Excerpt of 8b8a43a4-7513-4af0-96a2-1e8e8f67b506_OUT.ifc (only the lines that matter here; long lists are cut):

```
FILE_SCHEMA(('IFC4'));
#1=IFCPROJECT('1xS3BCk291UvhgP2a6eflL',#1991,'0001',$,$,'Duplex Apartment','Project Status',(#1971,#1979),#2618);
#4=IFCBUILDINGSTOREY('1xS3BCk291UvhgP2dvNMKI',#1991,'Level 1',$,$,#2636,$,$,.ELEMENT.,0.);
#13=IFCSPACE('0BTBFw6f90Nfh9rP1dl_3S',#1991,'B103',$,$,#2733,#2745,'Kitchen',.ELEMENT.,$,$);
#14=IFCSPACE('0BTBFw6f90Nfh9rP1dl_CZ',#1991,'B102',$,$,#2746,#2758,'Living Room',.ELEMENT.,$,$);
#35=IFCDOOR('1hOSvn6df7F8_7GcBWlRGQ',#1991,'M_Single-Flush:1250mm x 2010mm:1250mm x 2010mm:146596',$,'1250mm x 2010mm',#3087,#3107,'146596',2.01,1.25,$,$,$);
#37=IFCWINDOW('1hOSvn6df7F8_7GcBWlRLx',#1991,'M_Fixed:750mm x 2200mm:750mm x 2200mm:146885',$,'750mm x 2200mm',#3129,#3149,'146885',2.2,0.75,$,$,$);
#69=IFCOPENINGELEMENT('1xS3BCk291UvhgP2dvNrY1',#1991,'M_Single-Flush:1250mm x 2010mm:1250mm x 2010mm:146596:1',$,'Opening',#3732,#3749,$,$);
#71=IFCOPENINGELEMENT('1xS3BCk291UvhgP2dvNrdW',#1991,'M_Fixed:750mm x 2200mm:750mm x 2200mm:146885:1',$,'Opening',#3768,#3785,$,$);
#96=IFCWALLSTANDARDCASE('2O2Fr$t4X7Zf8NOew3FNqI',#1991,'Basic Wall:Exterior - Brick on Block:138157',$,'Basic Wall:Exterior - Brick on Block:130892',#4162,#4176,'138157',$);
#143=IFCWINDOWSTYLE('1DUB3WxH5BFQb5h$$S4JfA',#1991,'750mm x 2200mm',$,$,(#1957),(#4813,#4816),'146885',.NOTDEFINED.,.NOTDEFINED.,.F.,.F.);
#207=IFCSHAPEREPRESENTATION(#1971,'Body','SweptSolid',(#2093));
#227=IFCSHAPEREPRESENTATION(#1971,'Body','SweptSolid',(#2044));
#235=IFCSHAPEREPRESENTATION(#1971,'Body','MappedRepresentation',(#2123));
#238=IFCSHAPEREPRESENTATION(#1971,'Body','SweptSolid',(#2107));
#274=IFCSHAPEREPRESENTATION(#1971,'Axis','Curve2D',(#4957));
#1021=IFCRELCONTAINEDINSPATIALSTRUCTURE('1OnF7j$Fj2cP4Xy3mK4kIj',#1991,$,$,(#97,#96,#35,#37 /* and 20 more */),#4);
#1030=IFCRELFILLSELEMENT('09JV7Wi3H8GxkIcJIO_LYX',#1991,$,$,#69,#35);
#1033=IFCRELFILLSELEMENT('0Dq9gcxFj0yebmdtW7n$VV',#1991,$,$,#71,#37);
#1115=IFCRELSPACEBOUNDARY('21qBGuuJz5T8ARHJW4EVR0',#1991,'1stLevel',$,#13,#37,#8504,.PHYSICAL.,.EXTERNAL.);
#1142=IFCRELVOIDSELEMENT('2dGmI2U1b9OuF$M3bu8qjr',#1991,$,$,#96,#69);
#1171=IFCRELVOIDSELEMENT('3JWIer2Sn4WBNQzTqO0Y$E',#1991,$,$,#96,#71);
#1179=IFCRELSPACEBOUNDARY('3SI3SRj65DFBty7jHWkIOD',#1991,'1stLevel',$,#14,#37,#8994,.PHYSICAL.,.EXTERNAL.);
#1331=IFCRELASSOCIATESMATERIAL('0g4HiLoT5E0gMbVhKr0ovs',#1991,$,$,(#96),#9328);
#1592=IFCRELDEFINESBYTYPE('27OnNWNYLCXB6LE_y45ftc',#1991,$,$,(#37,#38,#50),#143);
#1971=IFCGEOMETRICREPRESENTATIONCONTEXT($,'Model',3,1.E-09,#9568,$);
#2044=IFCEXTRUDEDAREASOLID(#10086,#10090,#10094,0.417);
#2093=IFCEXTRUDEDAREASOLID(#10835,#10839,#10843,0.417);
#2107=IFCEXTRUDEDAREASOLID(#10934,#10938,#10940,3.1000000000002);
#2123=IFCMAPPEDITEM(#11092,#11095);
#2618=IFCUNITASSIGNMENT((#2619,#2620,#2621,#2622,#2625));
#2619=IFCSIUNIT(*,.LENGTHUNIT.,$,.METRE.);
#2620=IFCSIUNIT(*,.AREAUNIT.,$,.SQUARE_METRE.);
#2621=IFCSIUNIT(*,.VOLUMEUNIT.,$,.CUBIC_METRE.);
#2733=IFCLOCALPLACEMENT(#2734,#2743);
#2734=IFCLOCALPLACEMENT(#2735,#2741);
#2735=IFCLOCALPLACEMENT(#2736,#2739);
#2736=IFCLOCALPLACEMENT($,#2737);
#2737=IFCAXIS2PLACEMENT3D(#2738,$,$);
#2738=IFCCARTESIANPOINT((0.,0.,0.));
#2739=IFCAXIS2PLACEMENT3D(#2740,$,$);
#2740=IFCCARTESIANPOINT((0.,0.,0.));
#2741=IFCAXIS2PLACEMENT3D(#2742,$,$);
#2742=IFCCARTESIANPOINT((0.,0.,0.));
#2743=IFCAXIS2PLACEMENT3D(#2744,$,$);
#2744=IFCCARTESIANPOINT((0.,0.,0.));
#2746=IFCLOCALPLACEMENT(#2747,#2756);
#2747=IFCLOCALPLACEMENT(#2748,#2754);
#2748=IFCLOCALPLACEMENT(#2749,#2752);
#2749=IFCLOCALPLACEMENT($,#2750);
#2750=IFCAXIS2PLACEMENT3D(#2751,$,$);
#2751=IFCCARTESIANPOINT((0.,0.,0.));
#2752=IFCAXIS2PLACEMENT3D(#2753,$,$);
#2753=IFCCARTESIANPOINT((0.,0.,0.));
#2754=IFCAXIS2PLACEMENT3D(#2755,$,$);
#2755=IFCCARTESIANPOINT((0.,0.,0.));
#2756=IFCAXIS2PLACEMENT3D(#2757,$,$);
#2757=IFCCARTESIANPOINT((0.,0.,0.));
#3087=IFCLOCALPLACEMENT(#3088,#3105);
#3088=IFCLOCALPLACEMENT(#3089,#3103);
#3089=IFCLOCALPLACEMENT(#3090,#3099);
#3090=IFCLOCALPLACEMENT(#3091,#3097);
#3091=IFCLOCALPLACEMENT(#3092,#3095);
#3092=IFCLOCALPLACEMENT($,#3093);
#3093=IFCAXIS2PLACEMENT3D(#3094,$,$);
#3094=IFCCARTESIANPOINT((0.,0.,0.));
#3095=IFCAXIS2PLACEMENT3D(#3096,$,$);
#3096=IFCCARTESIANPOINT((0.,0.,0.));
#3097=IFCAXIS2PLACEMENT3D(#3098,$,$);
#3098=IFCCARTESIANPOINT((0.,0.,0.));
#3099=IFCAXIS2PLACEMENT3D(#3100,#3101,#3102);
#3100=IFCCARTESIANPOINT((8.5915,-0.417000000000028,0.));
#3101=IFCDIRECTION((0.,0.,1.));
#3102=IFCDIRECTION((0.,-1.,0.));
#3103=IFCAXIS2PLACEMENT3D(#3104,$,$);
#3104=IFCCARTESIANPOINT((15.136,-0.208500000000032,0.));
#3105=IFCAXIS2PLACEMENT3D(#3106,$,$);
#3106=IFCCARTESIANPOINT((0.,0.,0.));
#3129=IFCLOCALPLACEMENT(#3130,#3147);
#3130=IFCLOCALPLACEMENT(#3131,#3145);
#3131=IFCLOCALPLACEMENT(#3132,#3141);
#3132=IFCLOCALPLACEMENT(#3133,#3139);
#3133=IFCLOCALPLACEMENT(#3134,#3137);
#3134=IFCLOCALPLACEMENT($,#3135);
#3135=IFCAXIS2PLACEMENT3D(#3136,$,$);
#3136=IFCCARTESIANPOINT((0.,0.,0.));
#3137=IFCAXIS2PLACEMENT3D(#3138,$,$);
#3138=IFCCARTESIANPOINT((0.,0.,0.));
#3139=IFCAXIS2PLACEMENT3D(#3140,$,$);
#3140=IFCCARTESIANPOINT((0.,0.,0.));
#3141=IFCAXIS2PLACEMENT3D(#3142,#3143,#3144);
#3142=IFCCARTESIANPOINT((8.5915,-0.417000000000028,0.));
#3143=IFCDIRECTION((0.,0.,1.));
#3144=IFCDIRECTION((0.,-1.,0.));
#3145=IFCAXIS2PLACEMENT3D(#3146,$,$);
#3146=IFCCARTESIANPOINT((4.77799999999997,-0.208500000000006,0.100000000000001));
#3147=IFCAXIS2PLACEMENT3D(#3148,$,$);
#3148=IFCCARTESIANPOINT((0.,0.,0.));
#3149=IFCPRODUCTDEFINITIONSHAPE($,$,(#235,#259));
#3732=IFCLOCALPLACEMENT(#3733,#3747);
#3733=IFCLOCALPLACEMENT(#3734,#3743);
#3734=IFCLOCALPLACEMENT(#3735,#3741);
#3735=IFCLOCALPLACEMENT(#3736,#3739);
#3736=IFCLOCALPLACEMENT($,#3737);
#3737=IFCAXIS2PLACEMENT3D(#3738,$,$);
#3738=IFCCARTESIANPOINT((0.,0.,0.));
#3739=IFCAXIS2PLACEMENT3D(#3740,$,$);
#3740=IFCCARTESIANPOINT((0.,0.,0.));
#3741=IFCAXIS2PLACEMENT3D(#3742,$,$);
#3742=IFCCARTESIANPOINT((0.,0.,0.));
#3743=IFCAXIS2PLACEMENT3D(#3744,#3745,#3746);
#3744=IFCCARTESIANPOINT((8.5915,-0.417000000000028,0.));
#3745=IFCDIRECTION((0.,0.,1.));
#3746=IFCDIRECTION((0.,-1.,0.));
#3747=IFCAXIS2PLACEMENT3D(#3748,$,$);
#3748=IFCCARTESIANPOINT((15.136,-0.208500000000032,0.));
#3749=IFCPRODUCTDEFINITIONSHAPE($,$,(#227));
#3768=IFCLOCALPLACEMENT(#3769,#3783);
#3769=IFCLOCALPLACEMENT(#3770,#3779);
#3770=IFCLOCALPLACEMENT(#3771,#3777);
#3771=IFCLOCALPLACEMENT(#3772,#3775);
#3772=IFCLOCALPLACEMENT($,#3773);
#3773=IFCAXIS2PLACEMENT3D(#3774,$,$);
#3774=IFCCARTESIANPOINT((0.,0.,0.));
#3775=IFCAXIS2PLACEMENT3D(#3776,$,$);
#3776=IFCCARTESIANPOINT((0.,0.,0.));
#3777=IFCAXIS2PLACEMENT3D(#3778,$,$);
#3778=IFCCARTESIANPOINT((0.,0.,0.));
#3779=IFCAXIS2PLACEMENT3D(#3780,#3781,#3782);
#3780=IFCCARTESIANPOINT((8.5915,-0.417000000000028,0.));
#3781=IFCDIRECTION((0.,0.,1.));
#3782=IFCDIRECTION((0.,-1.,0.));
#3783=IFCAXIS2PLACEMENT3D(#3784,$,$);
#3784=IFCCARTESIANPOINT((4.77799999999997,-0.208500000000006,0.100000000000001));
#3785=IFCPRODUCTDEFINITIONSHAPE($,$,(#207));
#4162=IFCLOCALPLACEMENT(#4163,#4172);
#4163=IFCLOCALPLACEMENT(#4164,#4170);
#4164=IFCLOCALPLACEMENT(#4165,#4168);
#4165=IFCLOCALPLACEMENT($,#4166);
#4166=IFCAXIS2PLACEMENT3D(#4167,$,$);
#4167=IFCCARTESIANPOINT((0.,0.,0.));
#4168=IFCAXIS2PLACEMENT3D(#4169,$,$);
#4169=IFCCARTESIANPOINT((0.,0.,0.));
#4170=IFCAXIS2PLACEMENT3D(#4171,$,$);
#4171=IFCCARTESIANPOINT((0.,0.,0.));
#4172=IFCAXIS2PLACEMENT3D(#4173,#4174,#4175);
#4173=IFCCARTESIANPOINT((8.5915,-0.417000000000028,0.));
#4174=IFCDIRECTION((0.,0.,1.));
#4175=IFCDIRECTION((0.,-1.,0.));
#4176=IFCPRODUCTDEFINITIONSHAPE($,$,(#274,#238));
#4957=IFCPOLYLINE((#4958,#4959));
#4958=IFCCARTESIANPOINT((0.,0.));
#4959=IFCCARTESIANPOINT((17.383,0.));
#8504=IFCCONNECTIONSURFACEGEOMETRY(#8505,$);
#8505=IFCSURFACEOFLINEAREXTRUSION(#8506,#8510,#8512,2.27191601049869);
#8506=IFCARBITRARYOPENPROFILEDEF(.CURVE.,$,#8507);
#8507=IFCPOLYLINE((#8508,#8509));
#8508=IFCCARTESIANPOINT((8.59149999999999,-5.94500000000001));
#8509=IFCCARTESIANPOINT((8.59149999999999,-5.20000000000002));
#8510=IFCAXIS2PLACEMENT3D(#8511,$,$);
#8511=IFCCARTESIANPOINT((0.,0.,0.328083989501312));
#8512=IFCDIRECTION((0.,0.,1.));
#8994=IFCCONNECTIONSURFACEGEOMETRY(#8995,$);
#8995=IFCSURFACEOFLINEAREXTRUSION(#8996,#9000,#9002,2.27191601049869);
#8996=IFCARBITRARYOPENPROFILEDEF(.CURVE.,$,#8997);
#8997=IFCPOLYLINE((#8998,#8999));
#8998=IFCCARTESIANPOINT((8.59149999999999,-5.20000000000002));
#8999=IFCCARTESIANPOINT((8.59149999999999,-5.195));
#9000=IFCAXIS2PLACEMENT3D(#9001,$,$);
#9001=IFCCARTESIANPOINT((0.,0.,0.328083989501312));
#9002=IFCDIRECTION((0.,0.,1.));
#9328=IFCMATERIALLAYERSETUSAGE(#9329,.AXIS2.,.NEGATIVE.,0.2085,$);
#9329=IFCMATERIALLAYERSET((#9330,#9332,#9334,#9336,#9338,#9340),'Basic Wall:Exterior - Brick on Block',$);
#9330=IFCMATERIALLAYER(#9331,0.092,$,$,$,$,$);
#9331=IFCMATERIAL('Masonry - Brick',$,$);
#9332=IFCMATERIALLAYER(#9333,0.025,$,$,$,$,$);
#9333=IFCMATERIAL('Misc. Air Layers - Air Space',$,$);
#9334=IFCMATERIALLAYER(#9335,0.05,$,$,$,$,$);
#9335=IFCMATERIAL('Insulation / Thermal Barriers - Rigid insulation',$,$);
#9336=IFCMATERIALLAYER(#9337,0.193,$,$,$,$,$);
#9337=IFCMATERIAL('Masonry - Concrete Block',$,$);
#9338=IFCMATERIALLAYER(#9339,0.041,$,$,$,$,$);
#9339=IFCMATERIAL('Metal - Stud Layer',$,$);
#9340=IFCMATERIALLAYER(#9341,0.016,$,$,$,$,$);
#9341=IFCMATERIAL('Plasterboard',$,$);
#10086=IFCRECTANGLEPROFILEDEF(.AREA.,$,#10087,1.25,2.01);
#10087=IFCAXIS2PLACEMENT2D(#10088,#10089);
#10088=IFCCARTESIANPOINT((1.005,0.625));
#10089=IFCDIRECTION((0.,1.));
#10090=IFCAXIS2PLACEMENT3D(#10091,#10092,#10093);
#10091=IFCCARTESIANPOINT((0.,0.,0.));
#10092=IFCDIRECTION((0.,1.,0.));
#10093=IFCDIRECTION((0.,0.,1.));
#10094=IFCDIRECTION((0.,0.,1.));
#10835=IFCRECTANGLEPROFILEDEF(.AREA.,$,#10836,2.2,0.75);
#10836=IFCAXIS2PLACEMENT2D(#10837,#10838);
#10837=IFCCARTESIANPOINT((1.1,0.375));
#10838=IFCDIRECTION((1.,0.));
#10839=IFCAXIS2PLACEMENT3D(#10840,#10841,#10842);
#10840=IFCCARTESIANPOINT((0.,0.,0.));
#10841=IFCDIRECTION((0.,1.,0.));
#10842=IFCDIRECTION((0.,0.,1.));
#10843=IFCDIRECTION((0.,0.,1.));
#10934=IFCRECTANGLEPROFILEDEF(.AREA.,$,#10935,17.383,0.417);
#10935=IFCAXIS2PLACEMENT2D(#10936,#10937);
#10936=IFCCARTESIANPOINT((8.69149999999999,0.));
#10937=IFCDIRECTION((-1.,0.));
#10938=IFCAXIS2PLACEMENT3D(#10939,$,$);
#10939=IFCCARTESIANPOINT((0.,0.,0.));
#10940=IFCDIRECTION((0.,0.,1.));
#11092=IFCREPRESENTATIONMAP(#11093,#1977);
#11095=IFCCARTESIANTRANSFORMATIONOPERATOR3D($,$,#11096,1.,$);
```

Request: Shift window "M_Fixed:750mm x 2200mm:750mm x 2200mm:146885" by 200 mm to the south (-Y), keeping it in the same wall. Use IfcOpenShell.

```python
import numpy as np
import ifcopenshell
import ifcopenshell.api.geometry
import ifcopenshell.util.placement
import ifcopenshell.util.unit

model = ifcopenshell.open("8b8a43a4-7513-4af0-96a2-1e8e8f67b506_OUT.ifc")
unit_scale = ifcopenshell.util.unit.calculate_unit_scale(model)

window = model.by_guid("1hOSvn6df7F8_7GcBWlRLx")
opening = window.FillsVoids[0].RelatingOpeningElement
wall = opening.VoidsElements[0].RelatingBuildingElement

wall_matrix = ifcopenshell.util.placement.get_local_placement(wall.ObjectPlacement)
shift = wall_matrix[:3, 0] * 0.2 / unit_scale
before = ifcopenshell.util.placement.get_local_placement(window.ObjectPlacement)[:3, 3].copy()

# The window is not placed relative to its opening, so move both.
for product in (opening, window):
    matrix = ifcopenshell.util.placement.get_local_placement(product.ObjectPlacement)
    matrix[:3, 3] += shift
    ifcopenshell.api.geometry.edit_object_placement(model, product=product, matrix=matrix, is_si=False)

# Space boundary surfaces are stored in each space's coordinates; move them too.
for rel in window.ProvidesBoundaries:
    if not rel.ConnectionGeometry:
        continue
    surface = rel.ConnectionGeometry.SurfaceOnRelatingElement
    space_matrix = ifcopenshell.util.placement.get_local_placement(rel.RelatingSpace.ObjectPlacement)
    point = np.array(surface.Position.Location.Coordinates) + space_matrix[:3, :3].T @ shift
    surface.Position = model.createIfcAxis2Placement3D(
        model.createIfcCartesianPoint(point.tolist()), surface.Position.Axis, surface.Position.RefDirection
    )

after = ifcopenshell.util.placement.get_local_placement(window.ObjectPlacement)[:3, 3]
print("window moved by", (after - before).round(3) + 0.0)

model.write("8b8a43a4-7513-4af0-96a2-1e8e8f67b506_OUT_rev.ifc")
```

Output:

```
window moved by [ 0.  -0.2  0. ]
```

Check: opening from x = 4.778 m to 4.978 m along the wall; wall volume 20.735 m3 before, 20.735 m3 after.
